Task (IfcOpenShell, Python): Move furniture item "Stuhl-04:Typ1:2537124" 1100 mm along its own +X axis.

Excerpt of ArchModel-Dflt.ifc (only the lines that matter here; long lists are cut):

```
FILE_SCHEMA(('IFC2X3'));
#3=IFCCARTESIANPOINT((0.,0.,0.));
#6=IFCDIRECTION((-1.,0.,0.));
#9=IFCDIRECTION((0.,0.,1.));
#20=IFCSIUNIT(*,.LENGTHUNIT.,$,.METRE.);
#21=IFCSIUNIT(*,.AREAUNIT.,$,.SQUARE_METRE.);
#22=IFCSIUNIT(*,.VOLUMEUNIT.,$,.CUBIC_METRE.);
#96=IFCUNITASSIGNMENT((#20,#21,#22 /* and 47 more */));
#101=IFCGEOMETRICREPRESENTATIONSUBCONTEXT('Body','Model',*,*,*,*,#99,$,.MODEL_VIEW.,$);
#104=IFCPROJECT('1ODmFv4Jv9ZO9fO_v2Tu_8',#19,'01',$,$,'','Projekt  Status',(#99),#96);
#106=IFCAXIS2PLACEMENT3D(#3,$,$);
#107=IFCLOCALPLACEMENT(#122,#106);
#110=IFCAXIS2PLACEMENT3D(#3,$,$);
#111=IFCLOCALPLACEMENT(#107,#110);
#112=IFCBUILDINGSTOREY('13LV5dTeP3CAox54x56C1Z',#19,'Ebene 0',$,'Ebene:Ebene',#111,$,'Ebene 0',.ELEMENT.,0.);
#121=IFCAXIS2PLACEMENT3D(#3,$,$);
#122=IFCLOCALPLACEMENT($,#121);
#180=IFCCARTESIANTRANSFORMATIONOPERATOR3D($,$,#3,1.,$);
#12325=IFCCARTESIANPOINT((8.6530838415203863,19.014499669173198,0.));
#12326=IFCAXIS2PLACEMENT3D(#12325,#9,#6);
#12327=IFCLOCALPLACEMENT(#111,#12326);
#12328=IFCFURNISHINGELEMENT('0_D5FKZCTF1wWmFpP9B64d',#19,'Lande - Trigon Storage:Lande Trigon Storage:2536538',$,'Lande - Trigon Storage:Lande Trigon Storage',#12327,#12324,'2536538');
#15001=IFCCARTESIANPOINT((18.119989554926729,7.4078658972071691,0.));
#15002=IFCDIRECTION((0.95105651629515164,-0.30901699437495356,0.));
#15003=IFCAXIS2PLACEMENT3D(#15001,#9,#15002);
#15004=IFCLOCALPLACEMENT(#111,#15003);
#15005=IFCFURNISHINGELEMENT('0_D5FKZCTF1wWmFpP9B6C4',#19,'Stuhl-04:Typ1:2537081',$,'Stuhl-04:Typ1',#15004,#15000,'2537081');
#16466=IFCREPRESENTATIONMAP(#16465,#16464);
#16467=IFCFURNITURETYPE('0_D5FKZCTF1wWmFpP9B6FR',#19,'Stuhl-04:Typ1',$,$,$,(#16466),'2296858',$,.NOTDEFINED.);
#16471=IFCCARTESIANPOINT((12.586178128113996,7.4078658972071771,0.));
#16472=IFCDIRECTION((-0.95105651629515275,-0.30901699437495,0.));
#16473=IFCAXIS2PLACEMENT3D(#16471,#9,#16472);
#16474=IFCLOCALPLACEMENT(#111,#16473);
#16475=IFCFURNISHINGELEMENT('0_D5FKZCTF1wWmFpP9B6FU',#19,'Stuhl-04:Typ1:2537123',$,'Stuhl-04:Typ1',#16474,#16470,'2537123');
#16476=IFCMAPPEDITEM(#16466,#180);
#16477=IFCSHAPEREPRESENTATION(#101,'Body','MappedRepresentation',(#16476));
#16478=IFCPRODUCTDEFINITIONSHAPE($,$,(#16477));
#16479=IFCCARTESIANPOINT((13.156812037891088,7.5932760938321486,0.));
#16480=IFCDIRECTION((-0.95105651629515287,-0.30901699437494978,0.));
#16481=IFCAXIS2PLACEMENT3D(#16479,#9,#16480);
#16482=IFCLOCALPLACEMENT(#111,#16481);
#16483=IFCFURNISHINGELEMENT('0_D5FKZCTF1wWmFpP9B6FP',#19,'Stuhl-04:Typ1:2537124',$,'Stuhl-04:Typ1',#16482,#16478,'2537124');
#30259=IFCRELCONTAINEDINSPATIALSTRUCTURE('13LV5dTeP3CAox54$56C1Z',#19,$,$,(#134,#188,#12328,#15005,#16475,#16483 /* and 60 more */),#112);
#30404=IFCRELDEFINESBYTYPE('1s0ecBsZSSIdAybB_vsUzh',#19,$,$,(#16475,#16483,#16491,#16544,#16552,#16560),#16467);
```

```python
import ifcopenshell
import ifcopenshell.api.geometry
import ifcopenshell.util.placement
import ifcopenshell.util.unit

model = ifcopenshell.open("ArchModel-Dflt.ifc")
unit_scale = ifcopenshell.util.unit.calculate_unit_scale(model)

item = model.by_guid("0_D5FKZCTF1wWmFpP9B6FP")
matrix = ifcopenshell.util.placement.get_local_placement(item.ObjectPlacement)
matrix[:3, 3] += matrix[:3, 0] * 1.1 / unit_scale
ifcopenshell.api.geometry.edit_object_placement(model, product=item, matrix=matrix, is_si=False)

print(ifcopenshell.util.placement.get_local_placement(item.ObjectPlacement).round(3) + 0.0)

model.write("ArchModel-Dflt_v2.ifc")
```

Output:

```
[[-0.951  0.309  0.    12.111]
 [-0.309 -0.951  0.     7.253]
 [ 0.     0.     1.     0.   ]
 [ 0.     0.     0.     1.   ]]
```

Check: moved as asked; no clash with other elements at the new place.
